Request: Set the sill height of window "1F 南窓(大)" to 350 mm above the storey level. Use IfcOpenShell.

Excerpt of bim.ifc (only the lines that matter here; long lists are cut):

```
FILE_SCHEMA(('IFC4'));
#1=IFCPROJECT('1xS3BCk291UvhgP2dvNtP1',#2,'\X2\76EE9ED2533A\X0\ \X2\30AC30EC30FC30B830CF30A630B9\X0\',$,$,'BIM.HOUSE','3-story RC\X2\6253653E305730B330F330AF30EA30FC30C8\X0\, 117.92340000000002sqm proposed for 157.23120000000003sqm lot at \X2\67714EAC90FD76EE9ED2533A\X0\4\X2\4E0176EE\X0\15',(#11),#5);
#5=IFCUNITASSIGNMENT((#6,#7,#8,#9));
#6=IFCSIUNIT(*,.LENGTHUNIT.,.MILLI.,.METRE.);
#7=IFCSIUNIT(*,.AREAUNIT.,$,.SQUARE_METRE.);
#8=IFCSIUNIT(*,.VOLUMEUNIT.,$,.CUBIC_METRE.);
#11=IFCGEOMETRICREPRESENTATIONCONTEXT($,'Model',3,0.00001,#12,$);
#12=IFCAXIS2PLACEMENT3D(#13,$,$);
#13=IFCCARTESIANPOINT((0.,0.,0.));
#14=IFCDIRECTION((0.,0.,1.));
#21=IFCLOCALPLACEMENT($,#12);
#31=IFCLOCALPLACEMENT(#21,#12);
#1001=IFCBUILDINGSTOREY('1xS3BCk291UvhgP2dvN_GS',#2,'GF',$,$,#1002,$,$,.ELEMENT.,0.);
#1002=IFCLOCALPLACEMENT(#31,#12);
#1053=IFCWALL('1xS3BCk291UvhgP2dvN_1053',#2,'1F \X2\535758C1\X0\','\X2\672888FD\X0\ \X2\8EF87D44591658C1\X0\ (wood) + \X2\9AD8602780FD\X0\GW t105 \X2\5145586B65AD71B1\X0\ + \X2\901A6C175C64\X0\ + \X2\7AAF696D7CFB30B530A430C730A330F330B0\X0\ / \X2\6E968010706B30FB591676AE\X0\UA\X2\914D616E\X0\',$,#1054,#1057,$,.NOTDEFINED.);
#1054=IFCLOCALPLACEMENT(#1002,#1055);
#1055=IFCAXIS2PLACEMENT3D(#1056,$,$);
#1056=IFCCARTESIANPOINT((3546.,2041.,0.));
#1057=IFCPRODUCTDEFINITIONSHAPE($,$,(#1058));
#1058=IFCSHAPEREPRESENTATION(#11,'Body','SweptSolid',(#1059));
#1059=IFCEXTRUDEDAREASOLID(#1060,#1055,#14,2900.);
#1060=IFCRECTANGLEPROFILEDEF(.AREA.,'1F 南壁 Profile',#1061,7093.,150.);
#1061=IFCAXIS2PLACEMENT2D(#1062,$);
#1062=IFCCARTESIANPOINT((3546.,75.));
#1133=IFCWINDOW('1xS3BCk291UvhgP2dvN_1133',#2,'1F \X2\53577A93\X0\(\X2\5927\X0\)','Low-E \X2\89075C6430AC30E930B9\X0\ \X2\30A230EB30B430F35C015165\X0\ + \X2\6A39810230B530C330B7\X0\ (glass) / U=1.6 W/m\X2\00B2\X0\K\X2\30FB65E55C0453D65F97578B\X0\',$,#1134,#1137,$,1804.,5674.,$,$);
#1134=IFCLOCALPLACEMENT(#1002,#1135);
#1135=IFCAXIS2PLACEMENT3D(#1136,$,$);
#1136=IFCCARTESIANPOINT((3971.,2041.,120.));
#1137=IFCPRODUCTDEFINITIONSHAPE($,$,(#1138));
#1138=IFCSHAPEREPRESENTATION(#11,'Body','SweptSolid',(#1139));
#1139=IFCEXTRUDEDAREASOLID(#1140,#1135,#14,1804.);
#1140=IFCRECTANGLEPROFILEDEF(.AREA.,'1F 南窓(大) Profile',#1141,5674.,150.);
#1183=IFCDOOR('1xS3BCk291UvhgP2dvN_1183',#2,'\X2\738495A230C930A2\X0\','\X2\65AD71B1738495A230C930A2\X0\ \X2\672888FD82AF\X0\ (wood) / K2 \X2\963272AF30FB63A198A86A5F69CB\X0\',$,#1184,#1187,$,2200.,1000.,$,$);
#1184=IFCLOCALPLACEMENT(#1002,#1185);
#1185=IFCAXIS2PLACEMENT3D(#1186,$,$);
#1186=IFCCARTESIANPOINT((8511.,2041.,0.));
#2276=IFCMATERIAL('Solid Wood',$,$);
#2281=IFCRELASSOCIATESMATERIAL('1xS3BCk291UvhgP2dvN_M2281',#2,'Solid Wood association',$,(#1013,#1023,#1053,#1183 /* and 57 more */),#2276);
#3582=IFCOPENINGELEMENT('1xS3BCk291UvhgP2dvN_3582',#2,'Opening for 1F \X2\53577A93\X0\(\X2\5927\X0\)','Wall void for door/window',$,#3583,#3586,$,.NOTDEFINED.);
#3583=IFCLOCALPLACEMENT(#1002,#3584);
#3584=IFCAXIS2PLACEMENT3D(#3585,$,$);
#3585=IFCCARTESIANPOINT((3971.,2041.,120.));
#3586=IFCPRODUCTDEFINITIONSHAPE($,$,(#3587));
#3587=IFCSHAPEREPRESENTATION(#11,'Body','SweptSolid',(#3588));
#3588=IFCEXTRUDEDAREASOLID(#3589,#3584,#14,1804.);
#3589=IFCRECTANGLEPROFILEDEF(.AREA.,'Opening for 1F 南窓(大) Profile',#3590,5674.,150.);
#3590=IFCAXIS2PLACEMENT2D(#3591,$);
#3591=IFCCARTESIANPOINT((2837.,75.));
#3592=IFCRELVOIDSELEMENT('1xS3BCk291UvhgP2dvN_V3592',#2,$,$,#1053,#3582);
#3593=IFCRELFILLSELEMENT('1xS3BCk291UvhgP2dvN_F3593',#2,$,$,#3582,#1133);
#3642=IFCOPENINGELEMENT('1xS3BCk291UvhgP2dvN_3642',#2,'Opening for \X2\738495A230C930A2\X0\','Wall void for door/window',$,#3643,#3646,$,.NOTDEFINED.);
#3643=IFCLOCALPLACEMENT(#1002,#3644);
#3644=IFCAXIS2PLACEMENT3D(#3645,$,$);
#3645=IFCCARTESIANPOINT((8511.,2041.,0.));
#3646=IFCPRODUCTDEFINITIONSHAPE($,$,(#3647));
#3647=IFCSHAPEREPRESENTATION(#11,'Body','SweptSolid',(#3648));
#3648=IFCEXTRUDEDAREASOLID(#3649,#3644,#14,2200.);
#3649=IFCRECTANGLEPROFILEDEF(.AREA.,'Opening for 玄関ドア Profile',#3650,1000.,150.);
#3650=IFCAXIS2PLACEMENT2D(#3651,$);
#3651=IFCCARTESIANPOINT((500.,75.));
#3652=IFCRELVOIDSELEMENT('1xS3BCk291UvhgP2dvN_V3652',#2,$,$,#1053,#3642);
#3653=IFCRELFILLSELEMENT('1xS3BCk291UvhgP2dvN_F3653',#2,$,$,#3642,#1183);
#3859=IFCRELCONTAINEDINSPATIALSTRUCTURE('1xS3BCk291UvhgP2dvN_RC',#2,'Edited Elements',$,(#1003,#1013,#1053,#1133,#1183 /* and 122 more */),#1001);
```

```python
import numpy as np
import ifcopenshell
import ifcopenshell.api.geometry
import ifcopenshell.geom
import ifcopenshell.util.element
import ifcopenshell.util.placement
import ifcopenshell.util.shape
import ifcopenshell.util.unit

model = ifcopenshell.open("bim.ifc")
unit_scale = ifcopenshell.util.unit.calculate_unit_scale(model)

window = model.by_guid("1xS3BCk291UvhgP2dvN_1133")
opening = window.FillsVoids[0].RelatingOpeningElement
storey = ifcopenshell.util.element.get_container(window, ifc_class="IfcBuildingStorey")
level = ifcopenshell.util.placement.get_local_placement(storey.ObjectPlacement)[2, 3]

# The opening's origin need not be at the sill, so measure its lowest point.
shape = ifcopenshell.geom.create_shape(ifcopenshell.geom.settings(), opening)
bottom = ifcopenshell.util.shape.get_shape_bottom_elevation(shape, shape.geometry) / unit_scale
dz = level + 350.0 - bottom

shift = np.array([0.0, 0.0, dz])
# The window is not placed relative to its opening, so move both.
for product in (opening, window):
    matrix = ifcopenshell.util.placement.get_local_placement(product.ObjectPlacement)
    matrix[:3, 3] += shift
    ifcopenshell.api.geometry.edit_object_placement(model, product=product, matrix=matrix, is_si=False)

print(f"moved by {dz * unit_scale:+.3f} m")

model.write("bim_rev.ifc")
```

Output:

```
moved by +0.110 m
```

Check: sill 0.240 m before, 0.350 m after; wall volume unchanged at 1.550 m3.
